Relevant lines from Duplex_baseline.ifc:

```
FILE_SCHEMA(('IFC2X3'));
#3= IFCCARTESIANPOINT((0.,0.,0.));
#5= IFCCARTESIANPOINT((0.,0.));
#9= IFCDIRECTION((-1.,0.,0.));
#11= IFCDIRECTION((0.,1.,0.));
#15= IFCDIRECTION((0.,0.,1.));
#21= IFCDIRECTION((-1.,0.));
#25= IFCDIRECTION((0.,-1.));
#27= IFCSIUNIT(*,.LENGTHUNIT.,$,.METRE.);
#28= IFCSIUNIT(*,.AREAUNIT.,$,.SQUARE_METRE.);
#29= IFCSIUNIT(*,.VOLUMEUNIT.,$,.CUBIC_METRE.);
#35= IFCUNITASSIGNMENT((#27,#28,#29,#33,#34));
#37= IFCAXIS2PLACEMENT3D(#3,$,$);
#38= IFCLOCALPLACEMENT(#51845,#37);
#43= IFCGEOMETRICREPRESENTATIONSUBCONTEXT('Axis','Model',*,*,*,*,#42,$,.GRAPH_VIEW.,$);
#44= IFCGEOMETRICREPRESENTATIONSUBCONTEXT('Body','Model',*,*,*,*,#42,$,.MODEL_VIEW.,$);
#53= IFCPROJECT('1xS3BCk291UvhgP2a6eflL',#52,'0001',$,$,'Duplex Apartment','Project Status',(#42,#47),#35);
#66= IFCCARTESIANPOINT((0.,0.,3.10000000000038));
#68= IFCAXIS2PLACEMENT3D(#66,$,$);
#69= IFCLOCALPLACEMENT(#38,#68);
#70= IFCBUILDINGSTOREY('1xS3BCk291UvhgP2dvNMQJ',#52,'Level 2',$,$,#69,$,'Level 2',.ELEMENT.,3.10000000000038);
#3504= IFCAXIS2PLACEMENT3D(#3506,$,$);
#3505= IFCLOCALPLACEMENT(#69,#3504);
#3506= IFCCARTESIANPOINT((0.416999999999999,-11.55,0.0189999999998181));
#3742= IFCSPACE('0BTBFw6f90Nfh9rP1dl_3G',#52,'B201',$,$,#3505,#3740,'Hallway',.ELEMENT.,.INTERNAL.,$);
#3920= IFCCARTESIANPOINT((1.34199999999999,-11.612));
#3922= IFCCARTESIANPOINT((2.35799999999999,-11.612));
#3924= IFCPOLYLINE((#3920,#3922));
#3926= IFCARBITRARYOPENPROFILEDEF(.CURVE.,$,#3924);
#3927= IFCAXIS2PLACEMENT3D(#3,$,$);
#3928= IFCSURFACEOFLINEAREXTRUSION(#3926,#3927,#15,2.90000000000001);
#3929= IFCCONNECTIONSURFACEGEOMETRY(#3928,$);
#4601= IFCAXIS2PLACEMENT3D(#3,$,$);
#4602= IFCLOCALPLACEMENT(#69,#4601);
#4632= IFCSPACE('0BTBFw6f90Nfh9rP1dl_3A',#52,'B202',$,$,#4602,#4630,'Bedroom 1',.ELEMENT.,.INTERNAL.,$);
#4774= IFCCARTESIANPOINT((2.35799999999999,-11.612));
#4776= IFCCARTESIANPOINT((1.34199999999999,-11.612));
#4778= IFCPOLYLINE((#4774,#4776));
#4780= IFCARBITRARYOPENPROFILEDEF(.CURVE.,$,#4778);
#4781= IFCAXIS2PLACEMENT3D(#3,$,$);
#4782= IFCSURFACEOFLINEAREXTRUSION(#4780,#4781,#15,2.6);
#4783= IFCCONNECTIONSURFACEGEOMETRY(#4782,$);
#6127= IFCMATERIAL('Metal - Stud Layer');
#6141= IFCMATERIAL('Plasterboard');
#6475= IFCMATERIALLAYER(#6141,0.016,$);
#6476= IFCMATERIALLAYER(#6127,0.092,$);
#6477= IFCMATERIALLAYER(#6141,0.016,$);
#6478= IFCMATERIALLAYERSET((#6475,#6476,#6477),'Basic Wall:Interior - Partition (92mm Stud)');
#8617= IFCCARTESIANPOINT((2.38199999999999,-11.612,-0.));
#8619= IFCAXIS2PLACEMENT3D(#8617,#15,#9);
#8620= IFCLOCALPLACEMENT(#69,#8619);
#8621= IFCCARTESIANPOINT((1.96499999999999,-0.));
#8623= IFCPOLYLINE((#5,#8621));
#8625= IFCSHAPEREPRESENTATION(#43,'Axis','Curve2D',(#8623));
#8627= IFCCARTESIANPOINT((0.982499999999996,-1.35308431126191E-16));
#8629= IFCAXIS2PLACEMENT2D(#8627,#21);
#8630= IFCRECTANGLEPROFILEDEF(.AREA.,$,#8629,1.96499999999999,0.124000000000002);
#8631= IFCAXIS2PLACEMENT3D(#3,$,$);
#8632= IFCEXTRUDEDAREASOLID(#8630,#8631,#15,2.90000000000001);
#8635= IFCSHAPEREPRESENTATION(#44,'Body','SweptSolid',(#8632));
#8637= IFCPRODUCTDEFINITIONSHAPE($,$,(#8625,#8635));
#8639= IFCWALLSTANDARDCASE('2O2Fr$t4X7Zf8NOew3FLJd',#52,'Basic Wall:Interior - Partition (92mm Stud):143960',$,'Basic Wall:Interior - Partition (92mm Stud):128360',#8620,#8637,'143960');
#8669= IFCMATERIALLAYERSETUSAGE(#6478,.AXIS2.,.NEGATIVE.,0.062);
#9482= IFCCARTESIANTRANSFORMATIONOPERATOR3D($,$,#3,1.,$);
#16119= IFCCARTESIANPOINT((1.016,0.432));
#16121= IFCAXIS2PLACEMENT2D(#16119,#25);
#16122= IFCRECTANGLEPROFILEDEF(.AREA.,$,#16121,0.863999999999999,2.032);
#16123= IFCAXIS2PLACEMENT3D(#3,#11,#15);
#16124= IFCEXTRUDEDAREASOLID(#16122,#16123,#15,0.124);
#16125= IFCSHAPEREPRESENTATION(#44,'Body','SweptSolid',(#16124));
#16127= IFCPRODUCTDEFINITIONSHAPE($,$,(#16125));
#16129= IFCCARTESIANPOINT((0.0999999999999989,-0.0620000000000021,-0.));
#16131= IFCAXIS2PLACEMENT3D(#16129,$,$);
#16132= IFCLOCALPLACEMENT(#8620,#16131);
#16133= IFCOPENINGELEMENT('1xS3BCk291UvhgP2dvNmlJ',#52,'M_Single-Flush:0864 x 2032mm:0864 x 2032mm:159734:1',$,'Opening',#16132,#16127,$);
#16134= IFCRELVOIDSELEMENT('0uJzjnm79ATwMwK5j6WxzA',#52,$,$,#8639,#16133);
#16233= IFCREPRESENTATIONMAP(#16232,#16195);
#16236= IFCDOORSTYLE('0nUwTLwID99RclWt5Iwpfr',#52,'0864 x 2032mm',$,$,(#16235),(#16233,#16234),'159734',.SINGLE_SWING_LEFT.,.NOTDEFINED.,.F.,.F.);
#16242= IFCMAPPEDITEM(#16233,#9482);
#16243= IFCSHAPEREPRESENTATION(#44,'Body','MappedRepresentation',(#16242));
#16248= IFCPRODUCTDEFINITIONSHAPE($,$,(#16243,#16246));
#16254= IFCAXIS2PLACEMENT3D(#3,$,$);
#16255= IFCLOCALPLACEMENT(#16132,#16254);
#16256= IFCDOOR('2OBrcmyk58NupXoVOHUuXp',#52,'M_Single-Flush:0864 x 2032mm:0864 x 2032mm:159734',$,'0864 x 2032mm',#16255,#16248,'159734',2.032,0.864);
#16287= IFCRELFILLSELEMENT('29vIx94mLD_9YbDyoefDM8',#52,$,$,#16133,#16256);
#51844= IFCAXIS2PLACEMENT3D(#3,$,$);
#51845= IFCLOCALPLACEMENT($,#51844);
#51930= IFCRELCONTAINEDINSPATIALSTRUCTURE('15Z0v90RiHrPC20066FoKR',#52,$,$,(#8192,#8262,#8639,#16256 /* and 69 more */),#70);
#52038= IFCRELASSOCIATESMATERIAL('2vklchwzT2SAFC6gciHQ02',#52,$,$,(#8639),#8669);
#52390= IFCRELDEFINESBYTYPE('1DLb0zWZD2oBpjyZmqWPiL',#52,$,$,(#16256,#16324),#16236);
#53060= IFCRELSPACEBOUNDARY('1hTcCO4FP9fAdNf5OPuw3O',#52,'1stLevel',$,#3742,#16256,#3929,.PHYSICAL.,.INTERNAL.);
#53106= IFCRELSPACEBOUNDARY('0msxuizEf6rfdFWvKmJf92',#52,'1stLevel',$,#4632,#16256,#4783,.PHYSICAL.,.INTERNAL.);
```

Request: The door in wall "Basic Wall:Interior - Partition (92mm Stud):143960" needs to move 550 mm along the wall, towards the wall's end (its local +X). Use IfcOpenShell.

```python
import numpy as np
import ifcopenshell
import ifcopenshell.api.geometry
import ifcopenshell.util.placement
import ifcopenshell.util.unit

model = ifcopenshell.open("Duplex_baseline.ifc")
unit_scale = ifcopenshell.util.unit.calculate_unit_scale(model)

door = model.by_guid("2OBrcmyk58NupXoVOHUuXp")
opening = door.FillsVoids[0].RelatingOpeningElement
wall = opening.VoidsElements[0].RelatingBuildingElement

wall_matrix = ifcopenshell.util.placement.get_local_placement(wall.ObjectPlacement)
shift = wall_matrix[:3, 0] * 0.55 / unit_scale
before = ifcopenshell.util.placement.get_local_placement(door.ObjectPlacement)[:3, 3].copy()

# The door is placed relative to its opening, so it follows when the opening moves.
matrix = ifcopenshell.util.placement.get_local_placement(opening.ObjectPlacement)
matrix[:3, 3] += shift
ifcopenshell.api.geometry.edit_object_placement(
    model, product=opening, matrix=matrix, is_si=False, should_transform_children=True
)

# Space boundary surfaces are stored in each space's coordinates; move them too.
for rel in door.ProvidesBoundaries:
    if not rel.ConnectionGeometry:
        continue
    surface = rel.ConnectionGeometry.SurfaceOnRelatingElement
    space_matrix = ifcopenshell.util.placement.get_local_placement(rel.RelatingSpace.ObjectPlacement)
    point = np.array(surface.Position.Location.Coordinates) + space_matrix[:3, :3].T @ shift
    surface.Position = model.createIfcAxis2Placement3D(
        model.createIfcCartesianPoint(point.tolist()), surface.Position.Axis, surface.Position.RefDirection
    )

after = ifcopenshell.util.placement.get_local_placement(door.ObjectPlacement)[:3, 3]
print("door moved by", (after - before).round(3) + 0.0)

model.write("Duplex_baseline_updated.ifc")
```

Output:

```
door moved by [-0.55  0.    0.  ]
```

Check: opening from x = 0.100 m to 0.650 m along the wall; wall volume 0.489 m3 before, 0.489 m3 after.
